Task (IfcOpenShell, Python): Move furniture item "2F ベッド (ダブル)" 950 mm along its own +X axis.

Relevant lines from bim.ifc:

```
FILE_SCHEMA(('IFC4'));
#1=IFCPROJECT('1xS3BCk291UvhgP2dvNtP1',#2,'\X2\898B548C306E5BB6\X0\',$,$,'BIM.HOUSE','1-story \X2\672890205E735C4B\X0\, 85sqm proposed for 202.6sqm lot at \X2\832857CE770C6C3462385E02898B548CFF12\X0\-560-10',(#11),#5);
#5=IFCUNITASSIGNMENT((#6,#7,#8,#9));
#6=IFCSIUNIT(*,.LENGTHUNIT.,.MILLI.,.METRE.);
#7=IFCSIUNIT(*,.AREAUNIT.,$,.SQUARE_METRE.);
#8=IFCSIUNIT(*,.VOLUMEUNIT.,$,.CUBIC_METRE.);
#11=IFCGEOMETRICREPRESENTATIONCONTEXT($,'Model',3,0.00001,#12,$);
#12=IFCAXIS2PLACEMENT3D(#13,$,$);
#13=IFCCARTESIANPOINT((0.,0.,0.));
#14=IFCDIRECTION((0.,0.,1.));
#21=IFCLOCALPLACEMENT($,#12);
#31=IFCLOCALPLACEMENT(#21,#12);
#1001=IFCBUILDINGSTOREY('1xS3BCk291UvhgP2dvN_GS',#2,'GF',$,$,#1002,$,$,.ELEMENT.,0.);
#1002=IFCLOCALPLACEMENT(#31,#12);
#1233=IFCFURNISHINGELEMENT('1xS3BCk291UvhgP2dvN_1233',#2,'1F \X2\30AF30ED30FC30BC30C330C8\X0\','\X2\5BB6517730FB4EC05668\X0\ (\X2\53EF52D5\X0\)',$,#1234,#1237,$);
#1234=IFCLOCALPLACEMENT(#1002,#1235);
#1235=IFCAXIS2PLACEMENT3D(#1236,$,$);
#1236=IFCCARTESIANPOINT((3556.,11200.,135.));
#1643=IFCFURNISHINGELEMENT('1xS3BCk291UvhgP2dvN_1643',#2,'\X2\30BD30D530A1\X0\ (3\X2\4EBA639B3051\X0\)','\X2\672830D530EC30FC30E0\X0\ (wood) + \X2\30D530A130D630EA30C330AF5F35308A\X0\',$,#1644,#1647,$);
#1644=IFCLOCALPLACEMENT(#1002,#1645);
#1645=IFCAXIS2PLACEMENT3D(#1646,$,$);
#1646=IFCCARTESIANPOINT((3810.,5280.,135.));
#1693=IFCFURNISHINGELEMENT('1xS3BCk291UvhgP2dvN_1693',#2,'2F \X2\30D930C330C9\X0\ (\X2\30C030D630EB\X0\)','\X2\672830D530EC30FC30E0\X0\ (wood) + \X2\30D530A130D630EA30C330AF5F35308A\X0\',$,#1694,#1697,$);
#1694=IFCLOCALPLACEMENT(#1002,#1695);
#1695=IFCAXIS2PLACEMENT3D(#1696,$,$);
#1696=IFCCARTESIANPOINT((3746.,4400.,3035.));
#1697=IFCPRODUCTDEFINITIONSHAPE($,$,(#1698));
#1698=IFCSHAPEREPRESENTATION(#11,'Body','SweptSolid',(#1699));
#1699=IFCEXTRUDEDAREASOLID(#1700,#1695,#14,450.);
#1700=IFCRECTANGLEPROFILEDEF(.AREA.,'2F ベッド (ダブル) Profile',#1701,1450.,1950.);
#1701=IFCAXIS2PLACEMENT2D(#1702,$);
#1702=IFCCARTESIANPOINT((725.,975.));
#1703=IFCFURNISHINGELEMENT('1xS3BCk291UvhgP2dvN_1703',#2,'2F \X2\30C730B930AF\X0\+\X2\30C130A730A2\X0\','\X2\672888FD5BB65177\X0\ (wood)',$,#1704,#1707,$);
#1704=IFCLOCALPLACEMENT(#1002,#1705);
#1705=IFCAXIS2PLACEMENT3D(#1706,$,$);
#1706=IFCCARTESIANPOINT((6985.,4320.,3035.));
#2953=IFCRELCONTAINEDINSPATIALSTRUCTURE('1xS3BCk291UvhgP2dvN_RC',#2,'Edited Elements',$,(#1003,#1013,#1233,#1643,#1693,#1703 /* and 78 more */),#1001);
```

```python
import ifcopenshell
import ifcopenshell.api.geometry
import ifcopenshell.util.placement

model = ifcopenshell.open("bim.ifc")

item = model.by_id(1693)
matrix = ifcopenshell.util.placement.get_local_placement(item.ObjectPlacement)
matrix[:3, 3] += matrix[:3, 0] * 950.0
ifcopenshell.api.geometry.edit_object_placement(model, product=item, matrix=matrix, is_si=False)

print(ifcopenshell.util.placement.get_local_placement(item.ObjectPlacement).round(3) + 0.0)

model.write("bim_v2.ifc")
```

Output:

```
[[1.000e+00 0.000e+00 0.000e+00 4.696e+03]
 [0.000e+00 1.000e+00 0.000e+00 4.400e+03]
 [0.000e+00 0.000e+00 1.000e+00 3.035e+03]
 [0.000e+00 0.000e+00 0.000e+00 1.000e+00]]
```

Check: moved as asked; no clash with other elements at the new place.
